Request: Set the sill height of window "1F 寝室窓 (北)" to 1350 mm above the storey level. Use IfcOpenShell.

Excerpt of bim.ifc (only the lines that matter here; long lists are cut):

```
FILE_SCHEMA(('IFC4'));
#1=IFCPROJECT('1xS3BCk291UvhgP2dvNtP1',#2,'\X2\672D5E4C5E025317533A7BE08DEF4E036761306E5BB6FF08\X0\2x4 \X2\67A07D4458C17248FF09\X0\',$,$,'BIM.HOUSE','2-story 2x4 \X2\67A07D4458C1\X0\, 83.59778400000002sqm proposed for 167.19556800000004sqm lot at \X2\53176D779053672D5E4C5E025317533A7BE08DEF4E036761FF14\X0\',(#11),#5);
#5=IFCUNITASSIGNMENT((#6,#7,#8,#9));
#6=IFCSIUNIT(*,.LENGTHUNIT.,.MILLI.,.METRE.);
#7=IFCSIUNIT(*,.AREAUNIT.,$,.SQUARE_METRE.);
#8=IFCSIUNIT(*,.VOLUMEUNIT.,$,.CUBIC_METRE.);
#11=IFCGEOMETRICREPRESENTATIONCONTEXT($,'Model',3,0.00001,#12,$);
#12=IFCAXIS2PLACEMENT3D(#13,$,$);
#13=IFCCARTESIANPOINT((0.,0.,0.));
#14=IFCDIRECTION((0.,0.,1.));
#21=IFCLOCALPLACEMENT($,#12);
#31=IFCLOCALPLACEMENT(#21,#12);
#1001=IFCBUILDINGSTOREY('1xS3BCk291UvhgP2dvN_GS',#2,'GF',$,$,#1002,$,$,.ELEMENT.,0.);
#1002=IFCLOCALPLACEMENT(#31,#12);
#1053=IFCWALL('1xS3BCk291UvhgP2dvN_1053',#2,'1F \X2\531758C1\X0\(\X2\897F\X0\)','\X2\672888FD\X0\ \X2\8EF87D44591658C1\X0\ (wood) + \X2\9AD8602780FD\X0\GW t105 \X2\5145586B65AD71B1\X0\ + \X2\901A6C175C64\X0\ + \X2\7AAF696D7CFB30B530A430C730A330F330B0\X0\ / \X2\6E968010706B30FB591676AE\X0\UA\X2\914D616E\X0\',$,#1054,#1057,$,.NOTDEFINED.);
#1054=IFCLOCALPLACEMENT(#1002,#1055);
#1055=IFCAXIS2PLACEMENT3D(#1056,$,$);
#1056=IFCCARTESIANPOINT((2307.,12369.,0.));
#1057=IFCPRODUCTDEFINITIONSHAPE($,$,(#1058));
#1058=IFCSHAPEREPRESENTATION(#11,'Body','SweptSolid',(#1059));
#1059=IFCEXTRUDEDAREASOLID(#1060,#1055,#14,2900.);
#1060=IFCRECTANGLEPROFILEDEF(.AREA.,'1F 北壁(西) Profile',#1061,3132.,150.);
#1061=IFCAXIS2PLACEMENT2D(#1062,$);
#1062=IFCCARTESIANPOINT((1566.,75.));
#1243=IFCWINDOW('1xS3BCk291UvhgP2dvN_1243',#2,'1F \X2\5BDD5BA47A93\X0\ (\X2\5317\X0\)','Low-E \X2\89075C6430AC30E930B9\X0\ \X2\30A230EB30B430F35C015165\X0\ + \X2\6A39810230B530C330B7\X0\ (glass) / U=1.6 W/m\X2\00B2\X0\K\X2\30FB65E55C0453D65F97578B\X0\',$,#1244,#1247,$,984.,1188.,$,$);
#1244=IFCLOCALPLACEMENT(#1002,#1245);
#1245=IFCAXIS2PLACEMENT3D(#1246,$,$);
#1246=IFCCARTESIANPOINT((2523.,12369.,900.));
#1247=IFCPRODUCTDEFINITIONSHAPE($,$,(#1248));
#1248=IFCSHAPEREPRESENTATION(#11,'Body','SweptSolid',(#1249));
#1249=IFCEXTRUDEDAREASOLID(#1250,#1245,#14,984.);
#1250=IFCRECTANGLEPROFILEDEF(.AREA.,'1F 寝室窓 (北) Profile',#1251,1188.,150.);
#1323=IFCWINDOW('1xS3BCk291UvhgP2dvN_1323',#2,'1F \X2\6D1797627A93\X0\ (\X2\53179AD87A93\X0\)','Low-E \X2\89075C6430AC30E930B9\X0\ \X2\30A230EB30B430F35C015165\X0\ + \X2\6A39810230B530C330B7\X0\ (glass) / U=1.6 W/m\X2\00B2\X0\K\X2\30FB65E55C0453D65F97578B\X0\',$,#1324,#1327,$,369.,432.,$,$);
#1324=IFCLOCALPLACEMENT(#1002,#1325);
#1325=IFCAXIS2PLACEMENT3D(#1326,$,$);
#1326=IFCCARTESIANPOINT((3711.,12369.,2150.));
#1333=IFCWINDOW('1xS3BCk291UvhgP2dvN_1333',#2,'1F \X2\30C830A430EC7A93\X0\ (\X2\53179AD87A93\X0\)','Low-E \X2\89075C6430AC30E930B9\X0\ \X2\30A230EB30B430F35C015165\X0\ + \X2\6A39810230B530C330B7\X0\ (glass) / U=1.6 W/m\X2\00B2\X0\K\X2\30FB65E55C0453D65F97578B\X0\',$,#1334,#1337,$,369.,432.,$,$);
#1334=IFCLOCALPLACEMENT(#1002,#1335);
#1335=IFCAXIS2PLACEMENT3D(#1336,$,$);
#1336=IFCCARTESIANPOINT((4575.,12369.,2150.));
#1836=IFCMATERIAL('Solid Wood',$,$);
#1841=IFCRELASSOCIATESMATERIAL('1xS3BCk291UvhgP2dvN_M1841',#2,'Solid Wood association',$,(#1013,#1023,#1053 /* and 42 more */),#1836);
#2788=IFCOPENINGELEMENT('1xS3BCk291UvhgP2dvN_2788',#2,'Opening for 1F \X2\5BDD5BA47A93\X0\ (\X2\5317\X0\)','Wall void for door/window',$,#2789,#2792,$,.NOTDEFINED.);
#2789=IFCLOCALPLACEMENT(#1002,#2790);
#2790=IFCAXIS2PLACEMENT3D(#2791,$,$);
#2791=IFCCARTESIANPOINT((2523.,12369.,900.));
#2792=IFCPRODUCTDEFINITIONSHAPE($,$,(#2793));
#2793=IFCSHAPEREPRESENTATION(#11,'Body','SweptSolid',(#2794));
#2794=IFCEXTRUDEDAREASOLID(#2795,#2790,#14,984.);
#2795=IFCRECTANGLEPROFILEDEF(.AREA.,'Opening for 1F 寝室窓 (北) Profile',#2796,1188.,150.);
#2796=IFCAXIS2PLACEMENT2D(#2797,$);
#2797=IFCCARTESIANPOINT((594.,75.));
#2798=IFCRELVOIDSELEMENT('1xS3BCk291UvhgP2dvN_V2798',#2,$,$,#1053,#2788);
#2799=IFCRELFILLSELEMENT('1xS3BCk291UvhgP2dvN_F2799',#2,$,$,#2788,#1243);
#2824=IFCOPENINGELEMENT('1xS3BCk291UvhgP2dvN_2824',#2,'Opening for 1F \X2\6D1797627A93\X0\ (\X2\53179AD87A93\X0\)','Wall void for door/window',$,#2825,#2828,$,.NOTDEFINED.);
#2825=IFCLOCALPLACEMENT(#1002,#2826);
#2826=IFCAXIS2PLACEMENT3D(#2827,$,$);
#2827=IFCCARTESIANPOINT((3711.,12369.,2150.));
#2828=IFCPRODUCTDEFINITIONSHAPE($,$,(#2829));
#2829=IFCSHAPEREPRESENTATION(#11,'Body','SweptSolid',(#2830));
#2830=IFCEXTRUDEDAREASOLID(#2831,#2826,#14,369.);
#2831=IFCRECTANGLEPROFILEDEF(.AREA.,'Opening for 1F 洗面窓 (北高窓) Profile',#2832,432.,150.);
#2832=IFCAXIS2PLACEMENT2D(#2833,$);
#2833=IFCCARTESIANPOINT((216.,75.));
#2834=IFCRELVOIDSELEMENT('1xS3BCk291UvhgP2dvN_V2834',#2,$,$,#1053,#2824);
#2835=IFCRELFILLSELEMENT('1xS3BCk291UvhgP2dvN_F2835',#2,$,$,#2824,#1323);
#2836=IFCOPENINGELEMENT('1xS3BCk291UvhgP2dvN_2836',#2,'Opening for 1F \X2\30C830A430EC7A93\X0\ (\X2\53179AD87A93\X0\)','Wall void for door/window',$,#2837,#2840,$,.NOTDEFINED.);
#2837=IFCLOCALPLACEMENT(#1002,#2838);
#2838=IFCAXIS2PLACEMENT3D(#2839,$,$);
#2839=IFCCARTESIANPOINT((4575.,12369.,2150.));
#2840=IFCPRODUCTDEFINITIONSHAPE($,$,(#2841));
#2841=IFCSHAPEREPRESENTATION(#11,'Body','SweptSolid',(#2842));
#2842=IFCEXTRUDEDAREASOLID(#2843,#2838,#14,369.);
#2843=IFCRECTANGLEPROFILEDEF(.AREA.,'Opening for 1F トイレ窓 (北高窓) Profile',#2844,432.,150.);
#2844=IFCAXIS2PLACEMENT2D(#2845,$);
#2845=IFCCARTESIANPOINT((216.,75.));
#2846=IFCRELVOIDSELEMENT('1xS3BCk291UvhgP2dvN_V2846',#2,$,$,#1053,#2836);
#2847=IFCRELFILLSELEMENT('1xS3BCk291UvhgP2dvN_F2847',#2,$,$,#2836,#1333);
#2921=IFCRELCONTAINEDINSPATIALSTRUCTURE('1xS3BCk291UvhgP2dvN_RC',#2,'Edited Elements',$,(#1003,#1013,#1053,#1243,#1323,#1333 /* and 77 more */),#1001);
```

```python
import numpy as np
import ifcopenshell
import ifcopenshell.api.geometry
import ifcopenshell.geom
import ifcopenshell.util.element
import ifcopenshell.util.placement
import ifcopenshell.util.shape
import ifcopenshell.util.unit

model = ifcopenshell.open("bim.ifc")
unit_scale = ifcopenshell.util.unit.calculate_unit_scale(model)

window = model.by_guid("1xS3BCk291UvhgP2dvN_1243")
opening = window.FillsVoids[0].RelatingOpeningElement
storey = ifcopenshell.util.element.get_container(window, ifc_class="IfcBuildingStorey")
level = ifcopenshell.util.placement.get_local_placement(storey.ObjectPlacement)[2, 3]

# The opening's origin need not be at the sill, so measure its lowest point.
shape = ifcopenshell.geom.create_shape(ifcopenshell.geom.settings(), opening)
bottom = ifcopenshell.util.shape.get_shape_bottom_elevation(shape, shape.geometry) / unit_scale
dz = level + 1.35 / unit_scale - bottom

shift = np.array([0.0, 0.0, dz])
# The window is not placed relative to its opening, so move both.
for product in (opening, window):
    matrix = ifcopenshell.util.placement.get_local_placement(product.ObjectPlacement)
    matrix[:3, 3] += shift
    ifcopenshell.api.geometry.edit_object_placement(model, product=product, matrix=matrix, is_si=False)

print(f"moved by {dz * unit_scale:+.3f} m")

model.write("bim_v2.ifc")
```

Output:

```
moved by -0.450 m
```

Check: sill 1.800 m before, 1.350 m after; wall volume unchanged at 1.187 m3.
